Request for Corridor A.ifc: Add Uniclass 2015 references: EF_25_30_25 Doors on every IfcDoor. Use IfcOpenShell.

First a look at what the model holds.

```python
import ifcopenshell

model = ifcopenshell.open("Corridor A.ifc")
print(model.schema)
print("classifications:", [c.Name for c in model.by_type("IfcClassification")])
for ifc_class in ("IfcDoor", "IfcRoof", "IfcStair", "IfcWall", "IfcWindow"):
    print(ifc_class, len(model.by_type(ifc_class)))
```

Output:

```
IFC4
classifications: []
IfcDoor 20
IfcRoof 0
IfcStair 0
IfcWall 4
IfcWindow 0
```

```python
import ifcopenshell
import ifcopenshell.api.classification

model = ifcopenshell.open("Corridor A.ifc")

system = ifcopenshell.api.classification.add_classification(model, classification="Uniclass 2015")

codes = {
    "IfcDoor": ("EF_25_30_25", "Doors"),
}
for ifc_class, (code, name) in codes.items():
    products = model.by_type(ifc_class)
    ifcopenshell.api.classification.add_reference(
        model, products=products, classification=system, identification=code, name=name
    )
    print(code, len(products))

model.write("Corridor A_rev.ifc")
```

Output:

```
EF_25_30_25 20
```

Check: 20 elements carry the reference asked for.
